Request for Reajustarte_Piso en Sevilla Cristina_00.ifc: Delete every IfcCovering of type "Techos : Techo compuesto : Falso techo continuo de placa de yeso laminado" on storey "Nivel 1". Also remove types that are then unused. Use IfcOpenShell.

First a look at what the model holds.

```python
import ifcopenshell
import ifcopenshell.util.element

model = ifcopenshell.open("Reajustarte_Piso en Sevilla Cristina_00.ifc")
print(model.schema)
storey = next(s for s in model.by_type("IfcBuildingStorey") if s.Name == "Nivel 1")
coverings = [e for e in ifcopenshell.util.element.get_decomposition(storey) if e.is_a("IfcCovering")]
seen = {}
for e in coverings:
    element_type = ifcopenshell.util.element.get_type(e)
    name = element_type.Name if element_type not in (None, e) else None
    seen[name] = seen.get(name, 0) + 1
for name, count in sorted(seen.items(), key=str):
    print(count, "x", name)
```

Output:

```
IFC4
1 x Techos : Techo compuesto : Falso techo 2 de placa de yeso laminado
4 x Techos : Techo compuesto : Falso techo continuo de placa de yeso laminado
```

```python
import ifcopenshell
import ifcopenshell.api.root
import ifcopenshell.util.element

model = ifcopenshell.open("Reajustarte_Piso en Sevilla Cristina_00.ifc")

storey = next(s for s in model.by_type("IfcBuildingStorey") if s.Name == "Nivel 1")
coverings = [e for e in ifcopenshell.util.element.get_decomposition(storey) if e.is_a("IfcCovering")]
targets = [e for e in coverings if (t := ifcopenshell.util.element.get_type(e)) not in (None, e) and t.Name == "Techos : Techo compuesto : Falso techo continuo de placa de yeso laminado"]
types = {ifcopenshell.util.element.get_type(e) for e in targets} - {None, *targets}

for e in targets:
    ifcopenshell.api.root.remove_product(model, product=e)
print(len(targets), "removed")

unused = [t for t in types if not ifcopenshell.util.element.get_types(t)]
for t in unused:
    ifcopenshell.api.root.remove_product(model, product=t)
print(len(unused), "unused types removed")

model.write("Reajustarte_Piso en Sevilla Cristina_00_v2.ifc")
```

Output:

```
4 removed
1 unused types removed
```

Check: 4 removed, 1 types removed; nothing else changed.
